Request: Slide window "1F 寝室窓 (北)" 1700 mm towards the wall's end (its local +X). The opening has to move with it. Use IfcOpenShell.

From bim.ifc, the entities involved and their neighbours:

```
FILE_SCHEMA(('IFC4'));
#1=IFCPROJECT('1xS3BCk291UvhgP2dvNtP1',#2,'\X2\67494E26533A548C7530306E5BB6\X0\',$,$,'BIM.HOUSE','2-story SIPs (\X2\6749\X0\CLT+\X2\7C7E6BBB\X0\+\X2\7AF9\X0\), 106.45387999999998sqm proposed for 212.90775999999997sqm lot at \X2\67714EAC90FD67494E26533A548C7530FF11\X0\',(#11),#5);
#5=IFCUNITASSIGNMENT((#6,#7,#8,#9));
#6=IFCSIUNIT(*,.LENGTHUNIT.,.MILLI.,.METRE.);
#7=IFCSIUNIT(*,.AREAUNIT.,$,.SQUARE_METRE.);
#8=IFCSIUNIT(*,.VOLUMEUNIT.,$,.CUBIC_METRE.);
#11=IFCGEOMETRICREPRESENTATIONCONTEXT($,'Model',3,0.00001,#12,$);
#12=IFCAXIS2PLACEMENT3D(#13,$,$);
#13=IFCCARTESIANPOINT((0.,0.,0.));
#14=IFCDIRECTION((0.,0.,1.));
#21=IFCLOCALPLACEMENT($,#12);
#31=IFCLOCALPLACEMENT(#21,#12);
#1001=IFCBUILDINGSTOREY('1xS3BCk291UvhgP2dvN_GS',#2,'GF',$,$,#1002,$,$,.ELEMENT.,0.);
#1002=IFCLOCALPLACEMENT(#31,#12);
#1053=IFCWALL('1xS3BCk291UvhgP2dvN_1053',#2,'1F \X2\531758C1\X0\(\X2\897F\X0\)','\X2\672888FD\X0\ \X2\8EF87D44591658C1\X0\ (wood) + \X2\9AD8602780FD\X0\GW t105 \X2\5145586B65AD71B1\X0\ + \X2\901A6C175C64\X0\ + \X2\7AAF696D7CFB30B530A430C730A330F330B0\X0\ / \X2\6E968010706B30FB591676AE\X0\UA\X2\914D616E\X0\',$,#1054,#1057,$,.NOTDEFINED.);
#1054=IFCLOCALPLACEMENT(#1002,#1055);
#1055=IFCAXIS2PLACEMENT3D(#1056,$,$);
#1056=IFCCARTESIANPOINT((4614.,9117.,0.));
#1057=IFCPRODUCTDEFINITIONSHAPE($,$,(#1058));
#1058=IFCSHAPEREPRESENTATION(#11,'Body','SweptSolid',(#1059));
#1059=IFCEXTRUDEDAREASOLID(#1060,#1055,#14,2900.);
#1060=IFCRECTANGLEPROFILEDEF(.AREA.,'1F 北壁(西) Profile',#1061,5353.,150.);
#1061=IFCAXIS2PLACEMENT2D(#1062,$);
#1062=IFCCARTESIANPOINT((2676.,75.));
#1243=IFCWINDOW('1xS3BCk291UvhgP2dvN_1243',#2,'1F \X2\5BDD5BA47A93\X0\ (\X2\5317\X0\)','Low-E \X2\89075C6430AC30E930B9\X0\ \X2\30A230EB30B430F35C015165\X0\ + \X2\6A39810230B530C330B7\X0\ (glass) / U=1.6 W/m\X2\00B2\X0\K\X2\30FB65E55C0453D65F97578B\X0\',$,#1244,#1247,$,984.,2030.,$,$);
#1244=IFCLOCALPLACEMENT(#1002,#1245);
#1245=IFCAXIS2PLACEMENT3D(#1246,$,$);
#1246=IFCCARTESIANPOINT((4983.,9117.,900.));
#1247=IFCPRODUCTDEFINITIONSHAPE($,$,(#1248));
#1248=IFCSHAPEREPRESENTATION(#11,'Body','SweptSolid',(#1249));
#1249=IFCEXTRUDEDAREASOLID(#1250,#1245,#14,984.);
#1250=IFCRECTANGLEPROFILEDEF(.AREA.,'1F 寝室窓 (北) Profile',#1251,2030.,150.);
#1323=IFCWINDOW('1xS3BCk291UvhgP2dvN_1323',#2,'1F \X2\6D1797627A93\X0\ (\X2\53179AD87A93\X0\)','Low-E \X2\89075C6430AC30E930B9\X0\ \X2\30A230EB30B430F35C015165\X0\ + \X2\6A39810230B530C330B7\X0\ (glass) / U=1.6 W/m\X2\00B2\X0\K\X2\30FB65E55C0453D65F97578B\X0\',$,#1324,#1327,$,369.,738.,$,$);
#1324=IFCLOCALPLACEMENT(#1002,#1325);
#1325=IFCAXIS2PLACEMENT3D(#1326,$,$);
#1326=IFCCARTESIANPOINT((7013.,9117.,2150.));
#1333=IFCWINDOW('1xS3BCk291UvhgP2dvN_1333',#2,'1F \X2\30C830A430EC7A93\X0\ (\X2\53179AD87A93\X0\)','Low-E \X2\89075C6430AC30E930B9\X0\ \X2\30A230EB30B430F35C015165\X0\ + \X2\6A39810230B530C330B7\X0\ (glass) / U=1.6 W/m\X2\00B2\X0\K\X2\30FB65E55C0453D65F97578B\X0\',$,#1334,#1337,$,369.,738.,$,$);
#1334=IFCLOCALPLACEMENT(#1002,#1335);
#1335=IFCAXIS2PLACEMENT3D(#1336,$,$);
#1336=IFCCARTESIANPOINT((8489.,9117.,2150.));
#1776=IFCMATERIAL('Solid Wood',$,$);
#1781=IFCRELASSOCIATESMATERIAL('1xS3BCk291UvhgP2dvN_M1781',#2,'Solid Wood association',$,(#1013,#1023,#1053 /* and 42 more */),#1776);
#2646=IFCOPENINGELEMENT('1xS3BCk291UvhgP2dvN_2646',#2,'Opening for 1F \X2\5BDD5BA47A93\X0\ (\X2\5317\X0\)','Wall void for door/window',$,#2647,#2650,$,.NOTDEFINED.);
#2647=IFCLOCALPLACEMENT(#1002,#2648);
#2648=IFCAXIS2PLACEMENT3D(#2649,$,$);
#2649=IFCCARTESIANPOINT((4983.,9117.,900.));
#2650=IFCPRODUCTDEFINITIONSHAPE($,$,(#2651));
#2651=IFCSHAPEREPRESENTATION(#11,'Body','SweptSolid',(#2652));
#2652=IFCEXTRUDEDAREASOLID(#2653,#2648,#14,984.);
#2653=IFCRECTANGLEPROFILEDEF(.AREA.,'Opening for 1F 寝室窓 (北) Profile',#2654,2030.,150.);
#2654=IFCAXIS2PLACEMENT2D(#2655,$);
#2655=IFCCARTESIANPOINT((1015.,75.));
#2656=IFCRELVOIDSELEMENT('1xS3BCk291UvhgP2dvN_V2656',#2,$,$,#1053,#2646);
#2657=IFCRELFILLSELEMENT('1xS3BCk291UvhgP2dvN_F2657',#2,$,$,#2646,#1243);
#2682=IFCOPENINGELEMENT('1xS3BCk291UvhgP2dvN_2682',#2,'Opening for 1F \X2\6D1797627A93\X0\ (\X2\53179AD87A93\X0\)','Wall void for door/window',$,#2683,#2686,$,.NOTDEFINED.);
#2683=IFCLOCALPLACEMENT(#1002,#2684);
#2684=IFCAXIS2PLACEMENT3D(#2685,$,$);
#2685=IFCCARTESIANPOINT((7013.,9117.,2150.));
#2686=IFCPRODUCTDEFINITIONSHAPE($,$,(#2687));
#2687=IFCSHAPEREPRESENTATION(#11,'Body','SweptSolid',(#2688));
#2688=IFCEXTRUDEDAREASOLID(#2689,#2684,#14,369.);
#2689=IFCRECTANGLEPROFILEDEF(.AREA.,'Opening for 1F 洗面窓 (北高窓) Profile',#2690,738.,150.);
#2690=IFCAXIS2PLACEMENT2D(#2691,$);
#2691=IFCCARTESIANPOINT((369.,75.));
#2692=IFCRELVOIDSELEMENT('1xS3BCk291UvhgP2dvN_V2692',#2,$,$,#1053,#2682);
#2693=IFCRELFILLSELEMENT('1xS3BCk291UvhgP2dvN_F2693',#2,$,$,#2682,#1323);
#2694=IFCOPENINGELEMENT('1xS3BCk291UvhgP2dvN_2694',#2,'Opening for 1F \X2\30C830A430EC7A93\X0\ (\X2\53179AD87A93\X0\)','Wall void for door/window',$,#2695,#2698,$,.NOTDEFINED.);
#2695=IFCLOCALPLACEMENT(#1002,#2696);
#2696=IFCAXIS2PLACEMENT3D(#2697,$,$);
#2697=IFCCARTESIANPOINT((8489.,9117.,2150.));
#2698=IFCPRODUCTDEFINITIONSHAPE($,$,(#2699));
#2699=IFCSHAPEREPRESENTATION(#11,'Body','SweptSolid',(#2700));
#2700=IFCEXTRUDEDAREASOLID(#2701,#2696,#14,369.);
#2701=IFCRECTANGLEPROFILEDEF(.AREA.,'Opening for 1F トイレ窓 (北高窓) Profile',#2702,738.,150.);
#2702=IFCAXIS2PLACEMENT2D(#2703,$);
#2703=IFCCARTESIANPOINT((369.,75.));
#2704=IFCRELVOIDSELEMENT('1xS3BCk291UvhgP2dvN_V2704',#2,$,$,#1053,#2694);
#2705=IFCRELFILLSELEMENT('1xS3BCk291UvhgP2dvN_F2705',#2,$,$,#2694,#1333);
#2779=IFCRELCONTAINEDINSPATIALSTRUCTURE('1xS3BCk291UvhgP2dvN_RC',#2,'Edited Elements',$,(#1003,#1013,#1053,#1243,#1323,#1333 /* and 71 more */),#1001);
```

```python
import ifcopenshell
import ifcopenshell.api.geometry
import ifcopenshell.util.placement
import ifcopenshell.util.unit

model = ifcopenshell.open("bim.ifc")
unit_scale = ifcopenshell.util.unit.calculate_unit_scale(model)

window = model.by_id(1243)
opening = window.FillsVoids[0].RelatingOpeningElement
wall = opening.VoidsElements[0].RelatingBuildingElement

wall_matrix = ifcopenshell.util.placement.get_local_placement(wall.ObjectPlacement)
shift = wall_matrix[:3, 0] * 1.7 / unit_scale
before = ifcopenshell.util.placement.get_local_placement(window.ObjectPlacement)[:3, 3].copy()

# The window is not placed relative to its opening, so move both.
for product in (opening, window):
    matrix = ifcopenshell.util.placement.get_local_placement(product.ObjectPlacement)
    matrix[:3, 3] += shift
    ifcopenshell.api.geometry.edit_object_placement(model, product=product, matrix=matrix, is_si=False)

after = ifcopenshell.util.placement.get_local_placement(window.ObjectPlacement)[:3, 3]
print("window moved by", (after - before).round(3) + 0.0)

model.write("bim-out.ifc")
```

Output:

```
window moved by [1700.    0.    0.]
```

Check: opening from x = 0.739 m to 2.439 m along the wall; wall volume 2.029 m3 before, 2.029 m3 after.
